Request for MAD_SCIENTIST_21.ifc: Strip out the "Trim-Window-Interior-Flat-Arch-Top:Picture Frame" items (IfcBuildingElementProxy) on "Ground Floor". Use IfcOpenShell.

First a look at what the model holds.

```python
import ifcopenshell
import ifcopenshell.util.element

model = ifcopenshell.open("MAD_SCIENTIST_21.ifc")
print(model.schema)
storey = next(s for s in model.by_type("IfcBuildingStorey") if s.Name == "Ground Floor")
proxies = [e for e in ifcopenshell.util.element.get_decomposition(storey) if e.is_a("IfcBuildingElementProxy")]
seen = {}
for e in proxies:
    element_type = ifcopenshell.util.element.get_type(e)
    name = element_type.Name if element_type not in (None, e) else None
    seen[name] = seen.get(name, 0) + 1
for name, count in sorted(seen.items(), key=str):
    print(count, "x", name)
```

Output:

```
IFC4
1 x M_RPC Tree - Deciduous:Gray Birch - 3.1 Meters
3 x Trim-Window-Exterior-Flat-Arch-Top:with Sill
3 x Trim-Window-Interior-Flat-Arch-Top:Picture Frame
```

```python
import ifcopenshell
import ifcopenshell.api.root
import ifcopenshell.util.element

model = ifcopenshell.open("MAD_SCIENTIST_21.ifc")

storey = next(s for s in model.by_type("IfcBuildingStorey") if s.Name == "Ground Floor")
proxies = [e for e in ifcopenshell.util.element.get_decomposition(storey) if e.is_a("IfcBuildingElementProxy")]
targets = [e for e in proxies if (t := ifcopenshell.util.element.get_type(e)) not in (None, e) and t.Name == "Trim-Window-Interior-Flat-Arch-Top:Picture Frame"]

for e in targets:
    ifcopenshell.api.root.remove_product(model, product=e)
print(len(targets), "removed")

model.write("MAD_SCIENTIST_21_updated.ifc")
```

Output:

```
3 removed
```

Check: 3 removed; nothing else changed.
